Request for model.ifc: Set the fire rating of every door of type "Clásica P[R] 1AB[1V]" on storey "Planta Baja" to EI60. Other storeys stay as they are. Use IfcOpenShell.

First a look at what the model holds.

```python
import ifcopenshell
import ifcopenshell.util.element

model = ifcopenshell.open("model.ifc")
print(model.schema)
storey = next(s for s in model.by_type("IfcBuildingStorey") if s.Name == "Planta Baja")
doors = [e for e in ifcopenshell.util.element.get_decomposition(storey) if e.is_a("IfcDoor")]
seen = {}
for e in doors:
    element_type = ifcopenshell.util.element.get_type(e)
    key = (element_type.Name if element_type != e and element_type else None, ifcopenshell.util.element.get_pset(e, "Pset_DoorCommon", "FireRating"))
    seen[key] = seen.get(key, 0) + 1
for (name, value), count in sorted(seen.items(), key=str):
    print(count, "x", name, "|", value)
```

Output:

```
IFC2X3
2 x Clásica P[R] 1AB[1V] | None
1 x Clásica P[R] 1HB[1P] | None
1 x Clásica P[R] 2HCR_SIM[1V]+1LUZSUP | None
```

```python
import ifcopenshell
import ifcopenshell.api.pset
import ifcopenshell.util.element

model = ifcopenshell.open("model.ifc")

storey = next(s for s in model.by_type("IfcBuildingStorey") if s.Name == "Planta Baja")
doors = [e for e in ifcopenshell.util.element.get_decomposition(storey) if e.is_a("IfcDoor")]

count = 0
for e in doors:
    element_type = ifcopenshell.util.element.get_type(e)
    if element_type in (None, e) or element_type.Name != "Clásica P[R] 1AB[1V]":
        continue
    # add_pset returns the element's existing set when there is one.
    pset = ifcopenshell.api.pset.add_pset(model, product=e, name="Pset_DoorCommon")
    ifcopenshell.api.pset.edit_pset(model, pset=pset, properties={"FireRating": "EI60"})
    count += 1

print(count, "doors updated")

model.write("model_v2.ifc")
```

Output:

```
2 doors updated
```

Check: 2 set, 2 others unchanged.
